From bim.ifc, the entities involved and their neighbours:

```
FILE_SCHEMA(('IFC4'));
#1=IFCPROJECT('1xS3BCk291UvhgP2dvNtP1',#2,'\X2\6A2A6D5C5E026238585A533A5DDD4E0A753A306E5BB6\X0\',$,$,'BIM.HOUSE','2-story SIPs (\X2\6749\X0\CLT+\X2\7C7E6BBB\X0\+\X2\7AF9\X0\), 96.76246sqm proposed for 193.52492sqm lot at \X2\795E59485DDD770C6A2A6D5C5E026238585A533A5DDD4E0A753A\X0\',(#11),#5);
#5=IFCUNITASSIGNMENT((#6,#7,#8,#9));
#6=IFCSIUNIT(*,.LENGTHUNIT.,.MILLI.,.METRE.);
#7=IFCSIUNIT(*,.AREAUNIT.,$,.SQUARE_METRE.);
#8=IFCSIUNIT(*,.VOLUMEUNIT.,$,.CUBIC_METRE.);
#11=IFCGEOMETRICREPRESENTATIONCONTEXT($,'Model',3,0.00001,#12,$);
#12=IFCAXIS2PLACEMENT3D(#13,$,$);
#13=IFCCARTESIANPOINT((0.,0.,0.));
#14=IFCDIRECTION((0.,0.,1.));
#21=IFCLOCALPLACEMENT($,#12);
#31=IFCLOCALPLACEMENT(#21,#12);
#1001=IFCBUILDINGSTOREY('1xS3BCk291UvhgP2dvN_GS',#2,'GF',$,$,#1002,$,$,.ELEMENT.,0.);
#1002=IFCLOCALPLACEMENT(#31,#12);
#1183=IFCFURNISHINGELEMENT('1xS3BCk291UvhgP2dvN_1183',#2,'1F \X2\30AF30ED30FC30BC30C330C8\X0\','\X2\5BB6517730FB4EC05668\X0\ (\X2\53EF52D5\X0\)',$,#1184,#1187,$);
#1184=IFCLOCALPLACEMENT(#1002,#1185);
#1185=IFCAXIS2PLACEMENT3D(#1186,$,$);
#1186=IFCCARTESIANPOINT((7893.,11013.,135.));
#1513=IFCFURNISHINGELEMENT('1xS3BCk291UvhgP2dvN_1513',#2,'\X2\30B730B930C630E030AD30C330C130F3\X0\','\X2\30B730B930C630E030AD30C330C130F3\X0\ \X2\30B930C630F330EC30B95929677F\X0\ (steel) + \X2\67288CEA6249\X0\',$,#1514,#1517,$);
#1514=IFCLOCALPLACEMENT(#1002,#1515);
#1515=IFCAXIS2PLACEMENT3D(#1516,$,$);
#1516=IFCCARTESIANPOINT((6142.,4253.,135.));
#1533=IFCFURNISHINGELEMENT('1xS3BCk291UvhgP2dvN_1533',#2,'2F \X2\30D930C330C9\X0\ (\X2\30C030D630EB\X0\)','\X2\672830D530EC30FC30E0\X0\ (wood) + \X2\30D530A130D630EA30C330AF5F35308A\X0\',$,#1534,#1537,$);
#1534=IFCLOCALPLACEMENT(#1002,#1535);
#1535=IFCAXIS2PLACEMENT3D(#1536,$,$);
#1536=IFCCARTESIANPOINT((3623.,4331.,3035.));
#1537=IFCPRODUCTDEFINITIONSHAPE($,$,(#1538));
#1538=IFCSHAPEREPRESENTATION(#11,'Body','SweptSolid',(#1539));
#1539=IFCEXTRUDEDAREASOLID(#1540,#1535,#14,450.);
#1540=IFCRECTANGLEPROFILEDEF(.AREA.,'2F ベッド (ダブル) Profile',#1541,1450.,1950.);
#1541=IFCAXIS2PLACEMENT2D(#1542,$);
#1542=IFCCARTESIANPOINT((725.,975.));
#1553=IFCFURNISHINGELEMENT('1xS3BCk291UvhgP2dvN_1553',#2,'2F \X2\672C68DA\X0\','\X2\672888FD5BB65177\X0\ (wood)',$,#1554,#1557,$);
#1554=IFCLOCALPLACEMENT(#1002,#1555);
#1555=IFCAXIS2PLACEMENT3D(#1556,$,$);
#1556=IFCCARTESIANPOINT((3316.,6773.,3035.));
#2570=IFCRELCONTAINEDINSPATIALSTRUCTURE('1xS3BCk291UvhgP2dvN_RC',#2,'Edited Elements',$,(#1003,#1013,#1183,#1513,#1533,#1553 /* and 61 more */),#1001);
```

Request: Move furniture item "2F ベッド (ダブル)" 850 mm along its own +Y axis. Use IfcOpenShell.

```python
import ifcopenshell
import ifcopenshell.api.geometry
import ifcopenshell.util.placement
import ifcopenshell.util.unit

model = ifcopenshell.open("bim.ifc")
unit_scale = ifcopenshell.util.unit.calculate_unit_scale(model)

item = model.by_guid("1xS3BCk291UvhgP2dvN_1533")
matrix = ifcopenshell.util.placement.get_local_placement(item.ObjectPlacement)
matrix[:3, 3] += matrix[:3, 1] * 0.85 / unit_scale
ifcopenshell.api.geometry.edit_object_placement(model, product=item, matrix=matrix, is_si=False)

print(ifcopenshell.util.placement.get_local_placement(item.ObjectPlacement).round(3) + 0.0)

model.write("bim_rev.ifc")
```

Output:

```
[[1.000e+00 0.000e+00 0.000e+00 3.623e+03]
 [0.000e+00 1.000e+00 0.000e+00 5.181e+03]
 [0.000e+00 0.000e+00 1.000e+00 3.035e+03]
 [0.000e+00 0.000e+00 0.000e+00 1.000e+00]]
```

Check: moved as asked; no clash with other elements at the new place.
